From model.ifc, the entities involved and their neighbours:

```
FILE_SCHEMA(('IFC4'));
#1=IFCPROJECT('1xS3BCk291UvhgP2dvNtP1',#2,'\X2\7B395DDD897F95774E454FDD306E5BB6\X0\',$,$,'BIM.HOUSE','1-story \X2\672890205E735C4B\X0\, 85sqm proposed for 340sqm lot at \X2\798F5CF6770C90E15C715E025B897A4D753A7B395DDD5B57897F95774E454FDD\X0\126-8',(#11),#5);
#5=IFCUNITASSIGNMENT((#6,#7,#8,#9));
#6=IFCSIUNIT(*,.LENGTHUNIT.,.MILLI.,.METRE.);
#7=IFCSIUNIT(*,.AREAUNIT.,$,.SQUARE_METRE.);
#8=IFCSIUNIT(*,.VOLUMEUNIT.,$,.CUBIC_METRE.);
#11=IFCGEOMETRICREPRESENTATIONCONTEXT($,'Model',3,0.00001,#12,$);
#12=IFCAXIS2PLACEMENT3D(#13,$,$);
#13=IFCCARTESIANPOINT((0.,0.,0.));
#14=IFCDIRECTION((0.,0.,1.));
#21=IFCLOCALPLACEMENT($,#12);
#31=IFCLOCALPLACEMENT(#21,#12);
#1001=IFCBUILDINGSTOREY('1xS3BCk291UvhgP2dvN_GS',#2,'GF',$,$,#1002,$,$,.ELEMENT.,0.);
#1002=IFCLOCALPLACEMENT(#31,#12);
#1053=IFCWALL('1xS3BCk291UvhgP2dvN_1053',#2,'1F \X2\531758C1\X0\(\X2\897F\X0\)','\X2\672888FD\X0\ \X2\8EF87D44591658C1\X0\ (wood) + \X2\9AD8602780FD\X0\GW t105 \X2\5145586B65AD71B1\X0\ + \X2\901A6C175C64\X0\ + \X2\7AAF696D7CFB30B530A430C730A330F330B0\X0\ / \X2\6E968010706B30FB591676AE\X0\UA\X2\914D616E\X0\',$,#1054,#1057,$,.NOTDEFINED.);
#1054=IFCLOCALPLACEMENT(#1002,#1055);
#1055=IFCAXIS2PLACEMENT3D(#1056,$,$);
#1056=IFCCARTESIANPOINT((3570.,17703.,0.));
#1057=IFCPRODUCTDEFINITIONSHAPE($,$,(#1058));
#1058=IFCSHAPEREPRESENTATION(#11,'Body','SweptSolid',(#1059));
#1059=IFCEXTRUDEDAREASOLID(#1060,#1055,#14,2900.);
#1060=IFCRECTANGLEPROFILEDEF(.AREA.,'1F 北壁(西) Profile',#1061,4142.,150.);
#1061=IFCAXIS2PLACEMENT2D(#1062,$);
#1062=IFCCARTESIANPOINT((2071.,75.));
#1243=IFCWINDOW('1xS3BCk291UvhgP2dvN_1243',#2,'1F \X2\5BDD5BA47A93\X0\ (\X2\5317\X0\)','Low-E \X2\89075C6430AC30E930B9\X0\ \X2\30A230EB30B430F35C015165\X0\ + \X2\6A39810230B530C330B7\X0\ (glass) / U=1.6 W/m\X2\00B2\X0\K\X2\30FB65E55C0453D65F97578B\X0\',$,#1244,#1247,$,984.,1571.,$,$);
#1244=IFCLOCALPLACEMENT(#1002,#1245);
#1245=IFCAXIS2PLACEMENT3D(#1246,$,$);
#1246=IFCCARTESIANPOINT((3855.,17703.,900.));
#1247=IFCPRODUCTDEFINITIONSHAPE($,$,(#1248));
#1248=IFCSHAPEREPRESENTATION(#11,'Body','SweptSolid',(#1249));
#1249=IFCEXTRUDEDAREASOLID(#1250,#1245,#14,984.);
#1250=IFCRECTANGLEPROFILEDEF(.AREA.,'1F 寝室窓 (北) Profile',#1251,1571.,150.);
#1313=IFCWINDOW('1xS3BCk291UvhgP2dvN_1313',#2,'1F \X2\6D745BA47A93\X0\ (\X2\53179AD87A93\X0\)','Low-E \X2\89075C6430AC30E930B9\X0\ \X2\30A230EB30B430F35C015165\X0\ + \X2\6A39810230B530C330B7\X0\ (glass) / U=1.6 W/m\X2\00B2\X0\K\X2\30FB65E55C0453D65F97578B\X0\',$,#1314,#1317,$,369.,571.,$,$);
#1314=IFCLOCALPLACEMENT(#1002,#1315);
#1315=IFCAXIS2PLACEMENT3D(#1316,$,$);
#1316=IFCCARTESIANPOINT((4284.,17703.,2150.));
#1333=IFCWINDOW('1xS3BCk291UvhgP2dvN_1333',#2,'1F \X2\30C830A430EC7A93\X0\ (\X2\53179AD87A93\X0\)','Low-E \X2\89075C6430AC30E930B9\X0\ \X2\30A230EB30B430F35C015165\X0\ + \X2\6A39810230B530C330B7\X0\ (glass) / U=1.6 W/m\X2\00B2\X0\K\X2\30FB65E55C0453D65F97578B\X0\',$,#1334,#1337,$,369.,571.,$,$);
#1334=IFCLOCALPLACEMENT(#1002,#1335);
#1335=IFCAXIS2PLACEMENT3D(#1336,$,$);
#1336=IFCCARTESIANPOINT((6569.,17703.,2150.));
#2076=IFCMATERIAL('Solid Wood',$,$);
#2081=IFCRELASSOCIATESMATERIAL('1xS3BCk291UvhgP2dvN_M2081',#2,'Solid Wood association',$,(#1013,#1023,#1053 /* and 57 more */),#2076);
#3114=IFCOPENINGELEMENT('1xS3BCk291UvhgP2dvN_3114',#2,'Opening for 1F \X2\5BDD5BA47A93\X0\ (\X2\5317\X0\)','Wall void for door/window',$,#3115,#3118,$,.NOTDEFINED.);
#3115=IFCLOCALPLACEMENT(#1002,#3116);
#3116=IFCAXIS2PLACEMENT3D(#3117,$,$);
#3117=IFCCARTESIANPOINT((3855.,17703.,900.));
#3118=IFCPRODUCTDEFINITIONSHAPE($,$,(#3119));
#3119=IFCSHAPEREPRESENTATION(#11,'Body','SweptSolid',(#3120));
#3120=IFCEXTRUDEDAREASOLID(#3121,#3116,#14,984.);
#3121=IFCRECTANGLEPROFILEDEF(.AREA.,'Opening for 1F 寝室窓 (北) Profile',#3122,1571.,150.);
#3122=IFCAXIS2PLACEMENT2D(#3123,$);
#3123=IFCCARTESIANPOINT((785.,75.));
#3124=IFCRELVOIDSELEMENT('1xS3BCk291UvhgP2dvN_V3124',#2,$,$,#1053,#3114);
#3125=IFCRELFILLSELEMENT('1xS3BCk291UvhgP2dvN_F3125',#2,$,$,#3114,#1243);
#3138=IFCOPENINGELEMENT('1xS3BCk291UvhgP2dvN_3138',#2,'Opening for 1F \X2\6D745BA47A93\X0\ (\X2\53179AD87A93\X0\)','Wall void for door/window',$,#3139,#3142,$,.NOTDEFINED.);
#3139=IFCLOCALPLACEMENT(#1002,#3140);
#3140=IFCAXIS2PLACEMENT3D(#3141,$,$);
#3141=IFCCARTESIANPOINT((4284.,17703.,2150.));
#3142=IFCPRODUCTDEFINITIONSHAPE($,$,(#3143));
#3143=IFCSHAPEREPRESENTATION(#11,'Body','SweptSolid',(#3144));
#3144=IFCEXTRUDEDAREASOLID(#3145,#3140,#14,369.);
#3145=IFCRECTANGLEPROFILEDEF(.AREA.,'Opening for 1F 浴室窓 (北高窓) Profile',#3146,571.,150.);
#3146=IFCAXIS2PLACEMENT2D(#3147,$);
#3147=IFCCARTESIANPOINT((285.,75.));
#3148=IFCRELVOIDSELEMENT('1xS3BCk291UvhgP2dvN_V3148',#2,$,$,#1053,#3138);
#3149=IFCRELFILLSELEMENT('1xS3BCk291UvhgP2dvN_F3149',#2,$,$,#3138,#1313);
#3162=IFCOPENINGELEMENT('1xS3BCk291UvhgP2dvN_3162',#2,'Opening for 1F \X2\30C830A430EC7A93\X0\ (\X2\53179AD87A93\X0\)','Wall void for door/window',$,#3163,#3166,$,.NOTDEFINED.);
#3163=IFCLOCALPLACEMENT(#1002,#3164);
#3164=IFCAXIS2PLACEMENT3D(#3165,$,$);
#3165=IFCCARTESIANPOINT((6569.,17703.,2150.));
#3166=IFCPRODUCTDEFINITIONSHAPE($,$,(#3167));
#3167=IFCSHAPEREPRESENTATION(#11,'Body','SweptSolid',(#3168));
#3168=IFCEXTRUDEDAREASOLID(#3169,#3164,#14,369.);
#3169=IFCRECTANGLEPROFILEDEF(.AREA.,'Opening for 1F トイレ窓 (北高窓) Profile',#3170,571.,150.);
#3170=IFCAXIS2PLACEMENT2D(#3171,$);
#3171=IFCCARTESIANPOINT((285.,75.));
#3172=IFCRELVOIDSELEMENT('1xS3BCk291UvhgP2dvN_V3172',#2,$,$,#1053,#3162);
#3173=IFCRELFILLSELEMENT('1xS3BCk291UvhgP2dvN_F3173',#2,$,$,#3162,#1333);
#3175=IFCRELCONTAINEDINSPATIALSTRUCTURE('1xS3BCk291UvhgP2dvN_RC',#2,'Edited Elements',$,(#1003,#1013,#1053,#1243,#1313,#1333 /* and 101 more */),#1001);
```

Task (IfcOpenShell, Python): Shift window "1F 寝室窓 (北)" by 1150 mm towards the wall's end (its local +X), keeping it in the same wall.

```python
import ifcopenshell
import ifcopenshell.api.geometry
import ifcopenshell.util.placement
import ifcopenshell.util.unit

model = ifcopenshell.open("model.ifc")
unit_scale = ifcopenshell.util.unit.calculate_unit_scale(model)

window = model.by_guid("1xS3BCk291UvhgP2dvN_1243")
opening = window.FillsVoids[0].RelatingOpeningElement
wall = opening.VoidsElements[0].RelatingBuildingElement

wall_matrix = ifcopenshell.util.placement.get_local_placement(wall.ObjectPlacement)
shift = wall_matrix[:3, 0] * 1.15 / unit_scale
before = ifcopenshell.util.placement.get_local_placement(window.ObjectPlacement)[:3, 3].copy()

# The window is not placed relative to its opening, so move both.
for product in (opening, window):
    matrix = ifcopenshell.util.placement.get_local_placement(product.ObjectPlacement)
    matrix[:3, 3] += shift
    ifcopenshell.api.geometry.edit_object_placement(model, product=product, matrix=matrix, is_si=False)

after = ifcopenshell.util.placement.get_local_placement(window.ObjectPlacement)[:3, 3]
print("window moved by", (after - before).round(3) + 0.0)

model.write("model_v2.ifc")
```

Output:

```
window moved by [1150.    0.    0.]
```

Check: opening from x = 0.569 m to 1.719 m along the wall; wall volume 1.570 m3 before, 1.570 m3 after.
